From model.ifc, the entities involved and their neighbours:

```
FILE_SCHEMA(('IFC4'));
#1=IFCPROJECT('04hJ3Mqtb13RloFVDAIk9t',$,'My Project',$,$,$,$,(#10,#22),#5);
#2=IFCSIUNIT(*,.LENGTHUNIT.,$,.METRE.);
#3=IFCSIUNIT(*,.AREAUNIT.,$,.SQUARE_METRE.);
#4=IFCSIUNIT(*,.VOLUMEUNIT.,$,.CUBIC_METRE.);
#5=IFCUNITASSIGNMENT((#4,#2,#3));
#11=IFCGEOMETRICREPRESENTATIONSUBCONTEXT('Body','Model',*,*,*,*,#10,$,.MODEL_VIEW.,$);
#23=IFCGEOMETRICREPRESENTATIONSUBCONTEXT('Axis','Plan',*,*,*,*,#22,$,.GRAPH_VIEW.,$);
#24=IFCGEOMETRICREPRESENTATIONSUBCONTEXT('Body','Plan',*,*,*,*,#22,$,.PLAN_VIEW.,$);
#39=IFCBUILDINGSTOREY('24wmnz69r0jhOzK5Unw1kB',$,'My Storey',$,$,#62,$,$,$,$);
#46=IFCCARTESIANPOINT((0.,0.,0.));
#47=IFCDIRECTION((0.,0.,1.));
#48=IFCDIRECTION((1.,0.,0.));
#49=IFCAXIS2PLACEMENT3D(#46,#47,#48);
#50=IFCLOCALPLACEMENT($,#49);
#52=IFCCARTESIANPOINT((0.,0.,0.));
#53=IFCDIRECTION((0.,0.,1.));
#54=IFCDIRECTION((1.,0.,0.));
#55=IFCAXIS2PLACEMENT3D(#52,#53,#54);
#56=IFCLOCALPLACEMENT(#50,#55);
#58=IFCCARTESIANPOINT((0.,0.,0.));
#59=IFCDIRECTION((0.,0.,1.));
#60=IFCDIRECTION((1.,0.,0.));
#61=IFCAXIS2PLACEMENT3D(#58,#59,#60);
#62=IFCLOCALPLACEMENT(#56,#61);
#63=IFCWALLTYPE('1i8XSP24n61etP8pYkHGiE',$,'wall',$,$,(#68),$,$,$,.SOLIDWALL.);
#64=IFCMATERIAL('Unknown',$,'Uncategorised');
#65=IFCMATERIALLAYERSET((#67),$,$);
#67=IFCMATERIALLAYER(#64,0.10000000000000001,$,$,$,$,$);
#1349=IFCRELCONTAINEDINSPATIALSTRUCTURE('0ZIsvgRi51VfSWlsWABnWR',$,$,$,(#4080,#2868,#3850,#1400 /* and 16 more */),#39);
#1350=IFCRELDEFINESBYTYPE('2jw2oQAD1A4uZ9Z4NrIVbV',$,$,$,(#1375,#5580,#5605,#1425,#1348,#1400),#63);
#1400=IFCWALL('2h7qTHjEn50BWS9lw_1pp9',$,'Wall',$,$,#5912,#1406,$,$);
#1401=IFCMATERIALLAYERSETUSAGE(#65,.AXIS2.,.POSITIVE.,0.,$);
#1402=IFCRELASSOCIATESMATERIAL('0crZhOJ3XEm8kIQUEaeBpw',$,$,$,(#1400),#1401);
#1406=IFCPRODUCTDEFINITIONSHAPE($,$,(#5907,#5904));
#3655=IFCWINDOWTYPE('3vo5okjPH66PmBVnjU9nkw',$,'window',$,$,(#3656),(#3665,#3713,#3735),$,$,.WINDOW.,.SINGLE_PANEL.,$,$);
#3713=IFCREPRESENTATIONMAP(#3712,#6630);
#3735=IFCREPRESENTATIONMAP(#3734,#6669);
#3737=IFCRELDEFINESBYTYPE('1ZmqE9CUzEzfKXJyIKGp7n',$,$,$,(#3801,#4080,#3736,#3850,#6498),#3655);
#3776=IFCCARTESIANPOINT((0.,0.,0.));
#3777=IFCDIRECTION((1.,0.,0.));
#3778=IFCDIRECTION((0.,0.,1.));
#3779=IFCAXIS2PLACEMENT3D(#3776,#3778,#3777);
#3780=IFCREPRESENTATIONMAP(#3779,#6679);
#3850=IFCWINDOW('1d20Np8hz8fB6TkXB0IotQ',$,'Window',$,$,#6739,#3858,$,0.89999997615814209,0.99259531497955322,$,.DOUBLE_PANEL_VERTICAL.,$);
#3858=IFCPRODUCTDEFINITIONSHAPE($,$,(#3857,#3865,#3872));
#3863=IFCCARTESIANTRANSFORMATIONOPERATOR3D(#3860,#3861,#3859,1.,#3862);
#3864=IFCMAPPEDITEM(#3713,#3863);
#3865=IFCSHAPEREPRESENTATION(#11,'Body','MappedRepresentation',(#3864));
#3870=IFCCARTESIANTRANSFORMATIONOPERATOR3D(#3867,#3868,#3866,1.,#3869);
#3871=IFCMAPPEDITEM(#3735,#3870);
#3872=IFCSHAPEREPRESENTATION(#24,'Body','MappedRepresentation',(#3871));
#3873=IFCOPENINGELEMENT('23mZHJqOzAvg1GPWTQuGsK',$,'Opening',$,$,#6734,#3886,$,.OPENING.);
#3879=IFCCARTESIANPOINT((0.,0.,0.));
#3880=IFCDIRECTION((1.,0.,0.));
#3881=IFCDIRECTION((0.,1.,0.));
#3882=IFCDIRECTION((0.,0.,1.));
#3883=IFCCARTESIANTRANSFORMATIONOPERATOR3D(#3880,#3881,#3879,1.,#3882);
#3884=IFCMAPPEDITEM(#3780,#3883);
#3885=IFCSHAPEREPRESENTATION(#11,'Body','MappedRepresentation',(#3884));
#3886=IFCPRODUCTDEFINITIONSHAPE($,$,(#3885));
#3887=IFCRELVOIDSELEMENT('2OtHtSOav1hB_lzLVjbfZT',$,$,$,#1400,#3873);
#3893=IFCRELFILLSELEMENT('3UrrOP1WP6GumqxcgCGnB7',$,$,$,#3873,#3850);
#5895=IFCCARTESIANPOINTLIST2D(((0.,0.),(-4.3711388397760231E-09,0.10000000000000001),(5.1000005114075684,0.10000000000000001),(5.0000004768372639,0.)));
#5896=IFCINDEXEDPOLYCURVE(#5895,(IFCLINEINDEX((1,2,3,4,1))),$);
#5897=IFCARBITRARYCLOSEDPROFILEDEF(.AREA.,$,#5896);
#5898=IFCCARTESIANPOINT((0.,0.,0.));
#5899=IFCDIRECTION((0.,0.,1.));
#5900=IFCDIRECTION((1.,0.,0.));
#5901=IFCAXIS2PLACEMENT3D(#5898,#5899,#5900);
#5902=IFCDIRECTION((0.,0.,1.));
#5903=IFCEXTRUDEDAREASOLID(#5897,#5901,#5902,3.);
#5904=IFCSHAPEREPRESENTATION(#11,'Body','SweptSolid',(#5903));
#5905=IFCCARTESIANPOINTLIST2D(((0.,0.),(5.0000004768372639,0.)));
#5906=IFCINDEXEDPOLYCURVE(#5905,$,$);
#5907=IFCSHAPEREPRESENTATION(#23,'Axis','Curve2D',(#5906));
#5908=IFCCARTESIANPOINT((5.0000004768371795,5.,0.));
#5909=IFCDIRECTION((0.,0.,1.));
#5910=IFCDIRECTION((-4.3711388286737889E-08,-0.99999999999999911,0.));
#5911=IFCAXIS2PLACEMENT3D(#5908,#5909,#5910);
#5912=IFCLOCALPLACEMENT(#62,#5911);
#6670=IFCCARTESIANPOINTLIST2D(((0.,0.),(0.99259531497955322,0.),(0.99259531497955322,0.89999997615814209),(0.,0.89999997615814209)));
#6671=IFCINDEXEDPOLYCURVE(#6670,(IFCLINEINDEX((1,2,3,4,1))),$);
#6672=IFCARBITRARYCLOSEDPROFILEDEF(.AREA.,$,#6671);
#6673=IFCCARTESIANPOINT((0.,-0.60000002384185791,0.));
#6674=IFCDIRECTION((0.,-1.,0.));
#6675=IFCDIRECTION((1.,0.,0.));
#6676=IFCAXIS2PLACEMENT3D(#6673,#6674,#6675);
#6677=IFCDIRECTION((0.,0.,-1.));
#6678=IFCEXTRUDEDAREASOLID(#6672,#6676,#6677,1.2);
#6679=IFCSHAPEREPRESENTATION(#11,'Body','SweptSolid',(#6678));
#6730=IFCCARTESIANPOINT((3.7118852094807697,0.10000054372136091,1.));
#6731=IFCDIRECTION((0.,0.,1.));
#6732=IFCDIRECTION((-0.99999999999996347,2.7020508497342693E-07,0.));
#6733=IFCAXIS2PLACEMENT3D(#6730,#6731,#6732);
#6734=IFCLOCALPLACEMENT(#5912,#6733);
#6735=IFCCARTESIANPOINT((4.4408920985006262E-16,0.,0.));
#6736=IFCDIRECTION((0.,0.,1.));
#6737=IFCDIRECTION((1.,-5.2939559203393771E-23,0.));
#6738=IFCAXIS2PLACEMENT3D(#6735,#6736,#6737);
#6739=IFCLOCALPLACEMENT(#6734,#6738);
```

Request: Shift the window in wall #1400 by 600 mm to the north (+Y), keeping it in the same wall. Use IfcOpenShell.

```python
import ifcopenshell
import ifcopenshell.api.geometry
import ifcopenshell.util.placement
import ifcopenshell.util.unit

model = ifcopenshell.open("model.ifc")
unit_scale = ifcopenshell.util.unit.calculate_unit_scale(model)

window = model.by_guid("1d20Np8hz8fB6TkXB0IotQ")
opening = window.FillsVoids[0].RelatingOpeningElement
wall = opening.VoidsElements[0].RelatingBuildingElement

wall_matrix = ifcopenshell.util.placement.get_local_placement(wall.ObjectPlacement)
shift = wall_matrix[:3, 0] * -0.6 / unit_scale
before = ifcopenshell.util.placement.get_local_placement(window.ObjectPlacement)[:3, 3].copy()

# The window is placed relative to its opening, so it follows when the opening moves.
matrix = ifcopenshell.util.placement.get_local_placement(opening.ObjectPlacement)
matrix[:3, 3] += shift
ifcopenshell.api.geometry.edit_object_placement(
    model, product=opening, matrix=matrix, is_si=False, should_transform_children=True
)

after = ifcopenshell.util.placement.get_local_placement(window.ObjectPlacement)[:3, 3]
print("window moved by", (after - before).round(3) + 0.0)

model.write("model_rev.ifc")
```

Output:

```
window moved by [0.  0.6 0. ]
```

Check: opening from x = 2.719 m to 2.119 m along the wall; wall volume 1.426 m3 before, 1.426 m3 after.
